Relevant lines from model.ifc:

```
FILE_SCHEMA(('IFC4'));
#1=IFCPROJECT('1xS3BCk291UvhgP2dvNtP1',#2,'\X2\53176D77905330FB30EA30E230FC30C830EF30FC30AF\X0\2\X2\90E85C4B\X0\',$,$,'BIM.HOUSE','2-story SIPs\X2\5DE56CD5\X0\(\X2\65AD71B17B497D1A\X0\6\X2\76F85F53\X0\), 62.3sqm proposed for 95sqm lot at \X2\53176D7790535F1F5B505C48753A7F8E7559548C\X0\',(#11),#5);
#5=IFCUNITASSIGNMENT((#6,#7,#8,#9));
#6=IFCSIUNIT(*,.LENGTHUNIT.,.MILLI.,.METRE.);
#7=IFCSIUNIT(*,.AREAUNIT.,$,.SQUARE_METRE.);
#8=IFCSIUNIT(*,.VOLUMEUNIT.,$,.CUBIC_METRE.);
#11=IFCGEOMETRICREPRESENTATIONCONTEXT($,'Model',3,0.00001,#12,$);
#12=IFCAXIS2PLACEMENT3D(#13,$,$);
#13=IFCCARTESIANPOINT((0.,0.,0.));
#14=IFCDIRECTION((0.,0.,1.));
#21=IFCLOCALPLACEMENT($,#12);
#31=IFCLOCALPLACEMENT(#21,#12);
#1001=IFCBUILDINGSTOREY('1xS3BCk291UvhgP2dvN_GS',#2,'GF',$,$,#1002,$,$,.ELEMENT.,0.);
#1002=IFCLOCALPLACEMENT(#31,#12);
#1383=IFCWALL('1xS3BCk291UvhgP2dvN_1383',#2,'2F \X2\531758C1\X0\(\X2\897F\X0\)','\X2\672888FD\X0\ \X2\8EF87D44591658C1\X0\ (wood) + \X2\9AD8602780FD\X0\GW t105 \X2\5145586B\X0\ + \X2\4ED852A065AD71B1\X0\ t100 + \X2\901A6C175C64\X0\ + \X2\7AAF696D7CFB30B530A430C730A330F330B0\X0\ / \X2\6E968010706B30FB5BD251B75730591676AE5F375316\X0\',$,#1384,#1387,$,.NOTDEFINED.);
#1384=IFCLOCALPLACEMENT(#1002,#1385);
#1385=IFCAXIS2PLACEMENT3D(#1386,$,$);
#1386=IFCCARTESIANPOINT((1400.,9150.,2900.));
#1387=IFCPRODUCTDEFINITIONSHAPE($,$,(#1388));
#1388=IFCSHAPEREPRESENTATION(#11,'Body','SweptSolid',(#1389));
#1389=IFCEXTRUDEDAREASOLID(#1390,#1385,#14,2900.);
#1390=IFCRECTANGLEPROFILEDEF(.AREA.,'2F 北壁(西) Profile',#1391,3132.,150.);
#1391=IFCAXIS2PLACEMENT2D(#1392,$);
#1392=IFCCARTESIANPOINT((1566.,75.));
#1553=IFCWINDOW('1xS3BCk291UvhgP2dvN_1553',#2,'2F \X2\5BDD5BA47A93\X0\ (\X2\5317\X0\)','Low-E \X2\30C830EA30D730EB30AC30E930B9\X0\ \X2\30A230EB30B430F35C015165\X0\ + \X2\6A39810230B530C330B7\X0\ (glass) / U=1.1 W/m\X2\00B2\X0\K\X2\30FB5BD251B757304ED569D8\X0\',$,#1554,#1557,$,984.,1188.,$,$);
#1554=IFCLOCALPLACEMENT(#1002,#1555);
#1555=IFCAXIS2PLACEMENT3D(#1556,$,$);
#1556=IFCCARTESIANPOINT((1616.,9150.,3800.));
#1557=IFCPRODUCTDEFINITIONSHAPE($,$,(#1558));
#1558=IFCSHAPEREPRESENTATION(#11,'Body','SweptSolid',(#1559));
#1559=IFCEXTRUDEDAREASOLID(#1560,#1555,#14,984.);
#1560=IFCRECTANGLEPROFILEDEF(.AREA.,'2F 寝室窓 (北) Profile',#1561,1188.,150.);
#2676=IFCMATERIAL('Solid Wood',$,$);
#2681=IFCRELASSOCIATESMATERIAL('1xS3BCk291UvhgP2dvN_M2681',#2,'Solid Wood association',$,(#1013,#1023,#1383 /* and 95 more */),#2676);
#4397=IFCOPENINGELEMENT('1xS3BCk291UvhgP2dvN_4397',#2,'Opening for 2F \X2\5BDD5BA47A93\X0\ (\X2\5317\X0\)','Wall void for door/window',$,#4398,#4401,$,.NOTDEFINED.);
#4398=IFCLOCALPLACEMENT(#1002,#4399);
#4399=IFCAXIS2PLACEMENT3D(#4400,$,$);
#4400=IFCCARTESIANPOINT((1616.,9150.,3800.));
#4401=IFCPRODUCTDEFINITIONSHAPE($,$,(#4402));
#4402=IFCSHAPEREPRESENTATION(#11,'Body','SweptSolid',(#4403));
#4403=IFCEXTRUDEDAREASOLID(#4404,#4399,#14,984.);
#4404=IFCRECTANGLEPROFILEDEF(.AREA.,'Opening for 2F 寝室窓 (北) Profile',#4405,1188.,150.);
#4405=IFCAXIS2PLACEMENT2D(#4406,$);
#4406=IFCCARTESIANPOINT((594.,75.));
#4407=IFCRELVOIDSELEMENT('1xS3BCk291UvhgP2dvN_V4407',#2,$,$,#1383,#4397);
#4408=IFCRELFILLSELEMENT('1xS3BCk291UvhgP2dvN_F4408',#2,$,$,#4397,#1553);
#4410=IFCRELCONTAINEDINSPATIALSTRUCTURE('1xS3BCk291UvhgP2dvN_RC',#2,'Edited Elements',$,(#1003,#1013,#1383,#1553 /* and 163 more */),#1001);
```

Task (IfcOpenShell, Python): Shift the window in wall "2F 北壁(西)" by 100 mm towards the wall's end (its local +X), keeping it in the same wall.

```python
import ifcopenshell
import ifcopenshell.api.geometry
import ifcopenshell.util.placement
import ifcopenshell.util.unit

model = ifcopenshell.open("model.ifc")
unit_scale = ifcopenshell.util.unit.calculate_unit_scale(model)

window = model.by_guid("1xS3BCk291UvhgP2dvN_1553")
opening = window.FillsVoids[0].RelatingOpeningElement
wall = opening.VoidsElements[0].RelatingBuildingElement

wall_matrix = ifcopenshell.util.placement.get_local_placement(wall.ObjectPlacement)
shift = wall_matrix[:3, 0] * 0.1 / unit_scale
before = ifcopenshell.util.placement.get_local_placement(window.ObjectPlacement)[:3, 3].copy()

# The window is not placed relative to its opening, so move both.
for product in (opening, window):
    matrix = ifcopenshell.util.placement.get_local_placement(product.ObjectPlacement)
    matrix[:3, 3] += shift
    ifcopenshell.api.geometry.edit_object_placement(model, product=product, matrix=matrix, is_si=False)

after = ifcopenshell.util.placement.get_local_placement(window.ObjectPlacement)[:3, 3]
print("window moved by", (after - before).round(3) + 0.0)

model.write("model_v2.ifc")
```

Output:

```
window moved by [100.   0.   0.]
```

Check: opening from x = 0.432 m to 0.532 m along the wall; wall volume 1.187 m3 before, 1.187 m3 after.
